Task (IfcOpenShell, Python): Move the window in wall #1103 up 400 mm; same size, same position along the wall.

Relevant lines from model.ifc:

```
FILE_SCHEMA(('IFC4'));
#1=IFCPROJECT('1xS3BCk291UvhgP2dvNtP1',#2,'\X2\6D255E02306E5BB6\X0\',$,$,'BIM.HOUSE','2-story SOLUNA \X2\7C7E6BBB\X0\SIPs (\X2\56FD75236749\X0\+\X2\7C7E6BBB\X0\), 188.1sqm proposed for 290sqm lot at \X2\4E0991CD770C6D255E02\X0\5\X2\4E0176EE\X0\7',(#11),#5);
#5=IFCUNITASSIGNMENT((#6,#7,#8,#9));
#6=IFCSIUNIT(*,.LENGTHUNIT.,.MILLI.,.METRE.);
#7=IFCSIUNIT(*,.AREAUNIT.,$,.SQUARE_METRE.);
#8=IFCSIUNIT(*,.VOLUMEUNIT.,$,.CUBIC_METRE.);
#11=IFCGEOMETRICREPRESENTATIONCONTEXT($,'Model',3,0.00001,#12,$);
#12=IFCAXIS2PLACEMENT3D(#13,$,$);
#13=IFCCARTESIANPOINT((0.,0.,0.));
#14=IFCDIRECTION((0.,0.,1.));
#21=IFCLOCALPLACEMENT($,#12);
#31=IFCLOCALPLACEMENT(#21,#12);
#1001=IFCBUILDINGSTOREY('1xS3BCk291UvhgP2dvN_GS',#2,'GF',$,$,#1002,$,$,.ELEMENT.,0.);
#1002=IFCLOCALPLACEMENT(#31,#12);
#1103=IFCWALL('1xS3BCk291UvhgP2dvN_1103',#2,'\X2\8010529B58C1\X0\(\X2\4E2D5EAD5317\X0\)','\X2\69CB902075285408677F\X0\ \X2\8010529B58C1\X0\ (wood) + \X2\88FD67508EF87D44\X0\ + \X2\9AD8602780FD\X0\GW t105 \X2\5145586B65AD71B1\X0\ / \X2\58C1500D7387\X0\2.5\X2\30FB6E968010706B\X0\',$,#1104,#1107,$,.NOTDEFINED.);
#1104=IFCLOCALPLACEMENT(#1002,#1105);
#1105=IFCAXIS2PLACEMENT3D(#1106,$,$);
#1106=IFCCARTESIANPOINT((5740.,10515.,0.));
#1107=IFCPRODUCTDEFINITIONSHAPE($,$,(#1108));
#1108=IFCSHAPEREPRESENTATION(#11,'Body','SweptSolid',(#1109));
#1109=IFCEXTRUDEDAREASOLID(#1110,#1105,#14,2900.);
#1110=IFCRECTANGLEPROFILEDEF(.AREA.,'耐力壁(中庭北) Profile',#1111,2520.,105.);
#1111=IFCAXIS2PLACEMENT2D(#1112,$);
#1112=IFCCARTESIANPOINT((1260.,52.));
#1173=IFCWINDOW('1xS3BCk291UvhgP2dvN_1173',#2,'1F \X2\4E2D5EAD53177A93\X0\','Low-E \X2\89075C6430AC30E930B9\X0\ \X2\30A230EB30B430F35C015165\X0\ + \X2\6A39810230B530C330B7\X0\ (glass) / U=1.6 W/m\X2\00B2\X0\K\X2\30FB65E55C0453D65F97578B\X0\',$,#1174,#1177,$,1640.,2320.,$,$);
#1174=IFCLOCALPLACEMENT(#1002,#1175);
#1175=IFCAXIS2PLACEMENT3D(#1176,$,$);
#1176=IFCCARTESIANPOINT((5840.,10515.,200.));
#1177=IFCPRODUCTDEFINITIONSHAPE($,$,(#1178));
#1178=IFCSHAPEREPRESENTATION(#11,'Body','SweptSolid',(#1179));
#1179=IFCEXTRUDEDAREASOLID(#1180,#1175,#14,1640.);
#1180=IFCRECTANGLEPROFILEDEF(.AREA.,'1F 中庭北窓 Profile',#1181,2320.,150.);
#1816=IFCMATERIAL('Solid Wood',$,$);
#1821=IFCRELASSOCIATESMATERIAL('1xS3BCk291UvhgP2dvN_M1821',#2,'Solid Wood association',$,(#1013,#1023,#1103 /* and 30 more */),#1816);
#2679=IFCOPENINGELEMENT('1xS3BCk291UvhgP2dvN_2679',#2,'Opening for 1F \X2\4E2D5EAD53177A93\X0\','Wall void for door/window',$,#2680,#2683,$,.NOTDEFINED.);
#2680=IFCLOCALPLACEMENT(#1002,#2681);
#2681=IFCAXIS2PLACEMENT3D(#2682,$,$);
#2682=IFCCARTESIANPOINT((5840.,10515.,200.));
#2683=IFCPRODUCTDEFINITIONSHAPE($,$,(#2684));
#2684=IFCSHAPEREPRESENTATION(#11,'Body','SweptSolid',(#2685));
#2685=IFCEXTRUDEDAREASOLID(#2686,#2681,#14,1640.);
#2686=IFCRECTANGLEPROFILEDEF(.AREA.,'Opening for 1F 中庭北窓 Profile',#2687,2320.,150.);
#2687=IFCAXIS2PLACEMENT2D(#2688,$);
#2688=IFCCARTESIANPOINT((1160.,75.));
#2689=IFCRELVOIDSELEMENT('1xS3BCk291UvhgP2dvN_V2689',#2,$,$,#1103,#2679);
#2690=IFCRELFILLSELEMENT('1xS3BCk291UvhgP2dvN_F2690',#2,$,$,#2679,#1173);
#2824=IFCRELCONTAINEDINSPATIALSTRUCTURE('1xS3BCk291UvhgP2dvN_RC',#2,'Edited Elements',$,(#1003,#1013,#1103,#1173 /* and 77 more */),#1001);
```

```python
import numpy as np
import ifcopenshell
import ifcopenshell.api.geometry
import ifcopenshell.util.placement
import ifcopenshell.util.unit

model = ifcopenshell.open("model.ifc")
unit_scale = ifcopenshell.util.unit.calculate_unit_scale(model)

window = model.by_guid("1xS3BCk291UvhgP2dvN_1173")
opening = window.FillsVoids[0].RelatingOpeningElement
dz = 400.0

shift = np.array([0.0, 0.0, dz])
# The window is not placed relative to its opening, so move both.
for product in (opening, window):
    matrix = ifcopenshell.util.placement.get_local_placement(product.ObjectPlacement)
    matrix[:3, 3] += shift
    ifcopenshell.api.geometry.edit_object_placement(model, product=product, matrix=matrix, is_si=False)

print(f"moved by {dz * unit_scale:+.3f} m")

model.write("model_updated.ifc")
```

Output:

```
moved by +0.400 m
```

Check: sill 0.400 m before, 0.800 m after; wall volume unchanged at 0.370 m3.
